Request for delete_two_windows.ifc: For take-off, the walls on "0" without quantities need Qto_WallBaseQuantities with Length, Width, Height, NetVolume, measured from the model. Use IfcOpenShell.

First a look at what the model holds.

```python
import ifcopenshell
import ifcopenshell.util.element
import ifcopenshell.util.unit

model = ifcopenshell.open("delete_two_windows.ifc")
print(model.schema)
for unit_type in ("LENGTHUNIT", "AREAUNIT", "VOLUMEUNIT"):
    print(unit_type, ifcopenshell.util.unit.calculate_unit_scale(model, unit_type))
storey = next(s for s in model.by_type("IfcBuildingStorey") if s.Name == "0")
walls = [e for e in ifcopenshell.util.element.get_decomposition(storey) if e.is_a("IfcWall")]
for e in sorted(walls, key=lambda e: e.id()):
    print(e.id(), e.is_a(), e.Name, list(ifcopenshell.util.element.get_psets(e, qtos_only=True)), sep=" | ")
```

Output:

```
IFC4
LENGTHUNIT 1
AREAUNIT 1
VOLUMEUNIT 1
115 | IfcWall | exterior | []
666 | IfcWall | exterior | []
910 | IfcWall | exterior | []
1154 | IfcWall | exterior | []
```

```python
import ifcopenshell
import ifcopenshell.api.pset
import ifcopenshell.geom
import ifcopenshell.util.element
import ifcopenshell.util.shape
import ifcopenshell.util.unit

model = ifcopenshell.open("delete_two_windows.ifc")
unit_scale = ifcopenshell.util.unit.calculate_unit_scale(model)
volume_scale = ifcopenshell.util.unit.calculate_unit_scale(model, "VOLUMEUNIT")
settings = ifcopenshell.geom.settings()

storey = next(s for s in model.by_type("IfcBuildingStorey") if s.Name == "0")
walls = [e for e in ifcopenshell.util.element.get_decomposition(storey) if e.is_a("IfcWall")]

for e in sorted(walls, key=lambda e: e.id()):
    if ifcopenshell.util.element.get_psets(e, qtos_only=True, should_inherit=False):
        continue
    # Geometry comes back in metres, in the element's own axes.
    shape = ifcopenshell.geom.create_shape(settings, e)
    values = {
        "Length": ifcopenshell.util.shape.get_x(shape.geometry) / unit_scale,
        "Width": ifcopenshell.util.shape.get_y(shape.geometry) / unit_scale,
        "Height": ifcopenshell.util.shape.get_z(shape.geometry) / unit_scale,
        "NetVolume": ifcopenshell.util.shape.get_volume(shape.geometry) / volume_scale,
    }
    qto = ifcopenshell.api.pset.add_qto(model, product=e, name="Qto_WallBaseQuantities")
    ifcopenshell.api.pset.edit_qto(model, qto=qto, properties=values)
    print(e.id(), {k: round(v, 3) for k, v in values.items()})

model.write("delete_two_windows_v2.ifc")
```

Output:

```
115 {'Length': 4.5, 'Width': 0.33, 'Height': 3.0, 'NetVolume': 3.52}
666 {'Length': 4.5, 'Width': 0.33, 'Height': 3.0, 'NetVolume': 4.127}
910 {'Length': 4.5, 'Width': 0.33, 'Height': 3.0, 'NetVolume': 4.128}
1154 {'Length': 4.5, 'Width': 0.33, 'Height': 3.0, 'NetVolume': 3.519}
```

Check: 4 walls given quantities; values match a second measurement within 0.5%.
